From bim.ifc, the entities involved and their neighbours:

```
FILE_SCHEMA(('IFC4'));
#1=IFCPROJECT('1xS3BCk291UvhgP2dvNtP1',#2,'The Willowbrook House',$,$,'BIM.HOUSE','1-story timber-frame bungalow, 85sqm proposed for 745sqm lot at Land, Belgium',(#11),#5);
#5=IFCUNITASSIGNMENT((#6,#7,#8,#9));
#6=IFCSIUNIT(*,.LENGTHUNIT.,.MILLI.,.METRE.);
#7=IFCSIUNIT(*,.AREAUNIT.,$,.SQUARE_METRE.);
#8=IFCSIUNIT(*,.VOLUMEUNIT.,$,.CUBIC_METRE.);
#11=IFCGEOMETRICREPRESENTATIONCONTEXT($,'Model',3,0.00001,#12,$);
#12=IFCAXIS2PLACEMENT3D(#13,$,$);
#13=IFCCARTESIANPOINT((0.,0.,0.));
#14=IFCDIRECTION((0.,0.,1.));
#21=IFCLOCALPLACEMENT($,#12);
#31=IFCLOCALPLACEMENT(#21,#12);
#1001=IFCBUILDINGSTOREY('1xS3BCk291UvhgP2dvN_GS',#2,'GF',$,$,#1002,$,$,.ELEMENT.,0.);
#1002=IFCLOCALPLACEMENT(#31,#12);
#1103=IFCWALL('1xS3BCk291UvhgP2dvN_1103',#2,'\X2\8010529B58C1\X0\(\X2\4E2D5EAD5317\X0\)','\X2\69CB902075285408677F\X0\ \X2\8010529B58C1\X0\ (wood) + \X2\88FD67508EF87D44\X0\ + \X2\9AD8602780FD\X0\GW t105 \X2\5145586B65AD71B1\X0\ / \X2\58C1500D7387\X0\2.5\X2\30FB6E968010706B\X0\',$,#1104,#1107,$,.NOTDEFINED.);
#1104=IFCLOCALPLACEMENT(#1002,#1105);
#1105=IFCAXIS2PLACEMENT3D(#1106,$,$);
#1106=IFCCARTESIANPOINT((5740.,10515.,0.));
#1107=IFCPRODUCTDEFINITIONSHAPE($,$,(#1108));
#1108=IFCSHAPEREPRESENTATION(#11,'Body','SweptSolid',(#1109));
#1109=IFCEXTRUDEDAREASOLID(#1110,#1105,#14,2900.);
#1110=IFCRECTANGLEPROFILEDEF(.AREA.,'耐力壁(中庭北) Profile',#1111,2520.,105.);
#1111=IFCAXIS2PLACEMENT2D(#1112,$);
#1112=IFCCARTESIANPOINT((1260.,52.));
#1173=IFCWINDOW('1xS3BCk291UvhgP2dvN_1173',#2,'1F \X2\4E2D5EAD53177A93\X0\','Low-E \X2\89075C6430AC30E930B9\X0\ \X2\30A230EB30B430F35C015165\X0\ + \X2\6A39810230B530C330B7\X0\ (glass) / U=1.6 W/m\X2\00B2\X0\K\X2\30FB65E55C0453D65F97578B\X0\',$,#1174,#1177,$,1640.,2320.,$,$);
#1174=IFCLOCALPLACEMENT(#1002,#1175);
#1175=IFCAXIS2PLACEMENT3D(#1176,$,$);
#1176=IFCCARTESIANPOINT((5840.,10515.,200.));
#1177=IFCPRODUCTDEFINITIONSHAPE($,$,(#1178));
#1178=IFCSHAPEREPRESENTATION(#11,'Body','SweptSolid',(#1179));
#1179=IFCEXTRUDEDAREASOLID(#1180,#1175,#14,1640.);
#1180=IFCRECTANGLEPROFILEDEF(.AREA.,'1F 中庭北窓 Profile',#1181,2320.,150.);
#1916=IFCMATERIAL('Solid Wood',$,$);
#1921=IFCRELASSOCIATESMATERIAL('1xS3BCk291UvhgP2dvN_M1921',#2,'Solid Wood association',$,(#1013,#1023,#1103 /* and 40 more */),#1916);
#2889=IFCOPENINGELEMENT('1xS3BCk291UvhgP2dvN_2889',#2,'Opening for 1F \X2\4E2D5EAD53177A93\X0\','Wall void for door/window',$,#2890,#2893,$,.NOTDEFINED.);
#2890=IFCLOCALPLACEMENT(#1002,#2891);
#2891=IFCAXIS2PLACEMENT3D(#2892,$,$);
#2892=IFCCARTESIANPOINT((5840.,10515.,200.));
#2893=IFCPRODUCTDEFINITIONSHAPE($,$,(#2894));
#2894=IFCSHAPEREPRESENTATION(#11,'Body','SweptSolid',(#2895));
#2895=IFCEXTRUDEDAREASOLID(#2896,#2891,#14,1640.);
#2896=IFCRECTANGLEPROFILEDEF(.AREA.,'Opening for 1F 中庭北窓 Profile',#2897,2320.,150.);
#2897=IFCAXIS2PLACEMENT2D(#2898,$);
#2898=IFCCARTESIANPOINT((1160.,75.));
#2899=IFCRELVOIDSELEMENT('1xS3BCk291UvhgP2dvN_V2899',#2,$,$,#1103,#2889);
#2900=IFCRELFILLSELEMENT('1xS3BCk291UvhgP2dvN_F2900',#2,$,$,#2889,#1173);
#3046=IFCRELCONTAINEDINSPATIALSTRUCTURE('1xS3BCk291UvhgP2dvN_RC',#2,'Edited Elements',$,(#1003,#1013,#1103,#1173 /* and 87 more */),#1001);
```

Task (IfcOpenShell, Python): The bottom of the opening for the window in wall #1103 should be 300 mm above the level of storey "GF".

```python
import numpy as np
import ifcopenshell
import ifcopenshell.api.geometry
import ifcopenshell.geom
import ifcopenshell.util.element
import ifcopenshell.util.placement
import ifcopenshell.util.shape
import ifcopenshell.util.unit

model = ifcopenshell.open("bim.ifc")
unit_scale = ifcopenshell.util.unit.calculate_unit_scale(model)

window = model.by_guid("1xS3BCk291UvhgP2dvN_1173")
opening = window.FillsVoids[0].RelatingOpeningElement
storey = ifcopenshell.util.element.get_container(window, ifc_class="IfcBuildingStorey")
level = ifcopenshell.util.placement.get_local_placement(storey.ObjectPlacement)[2, 3]

# The opening's origin need not be at the sill, so measure its lowest point.
shape = ifcopenshell.geom.create_shape(ifcopenshell.geom.settings(), opening)
bottom = ifcopenshell.util.shape.get_shape_bottom_elevation(shape, shape.geometry) / unit_scale
dz = level + 300.0 - bottom

shift = np.array([0.0, 0.0, dz])
# The window is not placed relative to its opening, so move both.
for product in (opening, window):
    matrix = ifcopenshell.util.placement.get_local_placement(product.ObjectPlacement)
    matrix[:3, 3] += shift
    ifcopenshell.api.geometry.edit_object_placement(model, product=product, matrix=matrix, is_si=False)

print(f"moved by {dz * unit_scale:+.3f} m")

model.write("bim_v2.ifc")
```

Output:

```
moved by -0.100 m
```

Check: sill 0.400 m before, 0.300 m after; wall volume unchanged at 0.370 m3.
